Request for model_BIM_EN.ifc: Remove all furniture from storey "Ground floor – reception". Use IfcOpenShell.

First a look at what the model holds.

```python
import ifcopenshell
import ifcopenshell.util.element

model = ifcopenshell.open("model_BIM_EN.ifc")
print(model.schema)
storey = next(s for s in model.by_type("IfcBuildingStorey") if s.Name == "Ground floor – reception")
furniture = [e for e in ifcopenshell.util.element.get_decomposition(storey) if e.is_a("IfcFurnishingElement")]
seen = {}
for e in furniture:
    element_type = ifcopenshell.util.element.get_type(e)
    name = element_type.Name if element_type not in (None, e) else None
    seen[name] = seen.get(name, 0) + 1
for name, count in sorted(seen.items(), key=str):
    print(count, "x", name)
```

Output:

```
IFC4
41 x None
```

```python
import ifcopenshell
import ifcopenshell.api.root
import ifcopenshell.util.element

model = ifcopenshell.open("model_BIM_EN.ifc")

storey = next(s for s in model.by_type("IfcBuildingStorey") if s.Name == "Ground floor – reception")
furniture = [e for e in ifcopenshell.util.element.get_decomposition(storey) if e.is_a("IfcFurnishingElement")]

for e in furniture:
    ifcopenshell.api.root.remove_product(model, product=e)
print(len(furniture), "removed")

model.write("model_BIM_EN-out.ifc")
```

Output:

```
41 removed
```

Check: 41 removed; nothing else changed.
